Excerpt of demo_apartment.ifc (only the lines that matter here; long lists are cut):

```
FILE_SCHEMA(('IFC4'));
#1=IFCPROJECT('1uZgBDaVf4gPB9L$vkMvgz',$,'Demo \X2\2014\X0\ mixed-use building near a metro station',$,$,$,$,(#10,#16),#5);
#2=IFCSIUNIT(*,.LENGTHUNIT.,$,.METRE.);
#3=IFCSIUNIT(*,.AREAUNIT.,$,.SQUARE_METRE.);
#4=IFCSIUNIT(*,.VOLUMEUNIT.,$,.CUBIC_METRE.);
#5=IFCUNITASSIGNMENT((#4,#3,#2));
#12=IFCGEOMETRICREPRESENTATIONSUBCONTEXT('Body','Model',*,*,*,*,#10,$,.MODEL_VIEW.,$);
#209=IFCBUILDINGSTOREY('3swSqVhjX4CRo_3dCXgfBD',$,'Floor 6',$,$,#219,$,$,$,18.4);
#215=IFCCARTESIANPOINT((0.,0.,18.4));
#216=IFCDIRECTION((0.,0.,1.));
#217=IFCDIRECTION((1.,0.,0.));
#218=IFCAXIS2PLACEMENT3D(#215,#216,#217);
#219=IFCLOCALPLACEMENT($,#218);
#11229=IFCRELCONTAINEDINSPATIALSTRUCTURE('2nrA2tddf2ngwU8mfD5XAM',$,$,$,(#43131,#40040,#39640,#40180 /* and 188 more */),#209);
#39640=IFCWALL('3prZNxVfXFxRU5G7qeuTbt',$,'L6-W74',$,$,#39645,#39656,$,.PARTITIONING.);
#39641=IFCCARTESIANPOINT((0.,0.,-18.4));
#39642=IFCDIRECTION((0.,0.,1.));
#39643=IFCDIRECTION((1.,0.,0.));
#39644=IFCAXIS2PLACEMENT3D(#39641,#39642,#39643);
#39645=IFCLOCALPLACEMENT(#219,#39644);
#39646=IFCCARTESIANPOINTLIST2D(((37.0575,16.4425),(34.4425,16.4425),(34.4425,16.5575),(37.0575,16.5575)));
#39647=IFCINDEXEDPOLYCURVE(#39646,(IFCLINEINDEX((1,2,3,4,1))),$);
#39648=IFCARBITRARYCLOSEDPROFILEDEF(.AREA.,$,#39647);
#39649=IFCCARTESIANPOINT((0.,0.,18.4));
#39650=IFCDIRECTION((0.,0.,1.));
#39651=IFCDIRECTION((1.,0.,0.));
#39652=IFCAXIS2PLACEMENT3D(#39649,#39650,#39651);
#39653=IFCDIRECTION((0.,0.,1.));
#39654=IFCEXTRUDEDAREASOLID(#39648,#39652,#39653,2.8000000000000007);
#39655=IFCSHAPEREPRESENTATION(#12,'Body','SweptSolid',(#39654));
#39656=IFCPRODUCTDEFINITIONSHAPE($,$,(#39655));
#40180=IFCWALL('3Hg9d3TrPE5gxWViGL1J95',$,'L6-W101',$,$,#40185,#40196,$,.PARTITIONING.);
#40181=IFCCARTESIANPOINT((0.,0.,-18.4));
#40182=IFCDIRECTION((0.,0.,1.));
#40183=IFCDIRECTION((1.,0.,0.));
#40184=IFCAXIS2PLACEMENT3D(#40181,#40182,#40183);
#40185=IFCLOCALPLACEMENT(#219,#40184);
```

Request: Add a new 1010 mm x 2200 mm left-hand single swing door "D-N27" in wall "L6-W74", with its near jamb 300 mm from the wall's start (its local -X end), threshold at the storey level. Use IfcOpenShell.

```python
import numpy as np
import ifcopenshell
import ifcopenshell.api.feature
import ifcopenshell.api.geometry
import ifcopenshell.api.root
import ifcopenshell.api.spatial
import ifcopenshell.geom
import ifcopenshell.util.element
import ifcopenshell.util.placement
import ifcopenshell.util.representation
import ifcopenshell.util.shape
import ifcopenshell.util.unit

model = ifcopenshell.open("demo_apartment.ifc")
unit_scale = ifcopenshell.util.unit.calculate_unit_scale(model)
settings = ifcopenshell.geom.settings()


def volume(element):
    """Net volume in cubic metres, openings subtracted."""
    shape = ifcopenshell.geom.create_shape(settings, element)
    return ifcopenshell.util.shape.get_volume(shape.geometry)


wall = model.by_guid("3prZNxVfXFxRU5G7qeuTbt")
storey = ifcopenshell.util.element.get_container(wall, ifc_class="IfcBuildingStorey")
context = ifcopenshell.util.representation.get_context(model, "Model", "Body", "MODEL_VIEW")
before = volume(wall)

width, height, from_end, sill = 1.01, 2.2, 0.3, 0.0  # metres

# The wall runs along its own X axis, and the end named is its -X end.
wall_shape = ifcopenshell.geom.create_shape(settings, wall)
x, y, z = ifcopenshell.util.shape.get_vertices(wall_shape.geometry).T
start = x.min() + from_end
face, thickness = float(y.min()), float(y.max() - y.min())
wall_matrix = ifcopenshell.util.placement.get_local_placement(wall.ObjectPlacement)
level = ifcopenshell.util.placement.get_local_placement(storey.ObjectPlacement)[2, 3]


def in_wall(x, y):
    """Placement at x, y metres in the wall's axes, at sill height."""
    matrix = wall_matrix.copy()
    matrix[:, 3] = wall_matrix @ np.array([x / unit_scale, y / unit_scale, 0.0, 1.0])
    matrix[2, 3] = level + sill / unit_scale
    return matrix


# Opening: a box that overshoots both wall faces by 50 mm.
opening = ifcopenshell.api.root.create_entity(model, ifc_class="IfcOpeningElement", predefined_type="OPENING")
box = ifcopenshell.api.geometry.add_wall_representation(
    model, context=context, length=width, height=height, thickness=thickness + 0.1
)
ifcopenshell.api.geometry.assign_representation(model, product=opening, representation=box)
ifcopenshell.api.geometry.edit_object_placement(model, product=opening, matrix=in_wall(start, face - 0.05), is_si=False)
ifcopenshell.api.feature.add_feature(model, feature=opening, element=wall)

door = ifcopenshell.api.root.create_entity(model, ifc_class="IfcDoor", name="D-N27", predefined_type="DOOR")
door.OverallWidth, door.OverallHeight = width / unit_scale, height / unit_scale
door.OperationType = "SINGLE_SWING_LEFT"
body = ifcopenshell.api.geometry.add_door_representation(
    model,
    context=context,
    overall_width=door.OverallWidth,
    overall_height=door.OverallHeight,
    operation_type="SINGLE_SWING_LEFT",
    lining_properties={"LiningDepth": thickness / unit_scale, "ThresholdDepth": thickness / unit_scale},
)
ifcopenshell.api.geometry.assign_representation(model, product=door, representation=body)
ifcopenshell.api.spatial.assign_container(model, products=[door], relating_structure=storey)
ifcopenshell.api.feature.add_filling(model, opening=opening, element=door)

# The lining spans the wall, so the door starts at the wall face.
ifcopenshell.api.geometry.edit_object_placement(model, product=door, matrix=in_wall(start, face), is_si=False)

after = volume(wall)

print(f"wall volume {before:.3f} -> {after:.3f} m3")

model.write("demo_apartment_updated.ifc")
```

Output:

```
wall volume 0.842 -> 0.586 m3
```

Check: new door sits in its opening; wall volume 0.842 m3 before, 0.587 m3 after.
